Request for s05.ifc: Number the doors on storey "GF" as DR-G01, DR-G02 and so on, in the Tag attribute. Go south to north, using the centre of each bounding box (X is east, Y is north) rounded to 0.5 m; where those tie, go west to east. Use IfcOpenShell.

First a look at what the model holds.

```python
import ifcopenshell
import ifcopenshell.util.element
import ifcopenshell.util.placement

model = ifcopenshell.open("s05.ifc")
print(model.schema)
storey = next(s for s in model.by_type("IfcBuildingStorey") if s.Name == "GF")
doors = [e for e in ifcopenshell.util.element.get_decomposition(storey) if e.is_a("IfcDoor")]
for e in sorted(doors, key=lambda e: e.id()):
    origin = ifcopenshell.util.placement.get_local_placement(e.ObjectPlacement)[:3, 3]
    print(e.id(), e.Tag, e.Name, origin.round(2) + 0.0, sep=" | ")
```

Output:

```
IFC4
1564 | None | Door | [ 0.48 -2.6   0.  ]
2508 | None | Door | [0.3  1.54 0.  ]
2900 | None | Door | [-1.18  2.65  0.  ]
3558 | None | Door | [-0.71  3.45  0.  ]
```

```python
import ifcopenshell
import ifcopenshell.geom
import ifcopenshell.util.element
import ifcopenshell.util.shape

model = ifcopenshell.open("s05.ifc")
settings = ifcopenshell.geom.settings()
settings.set("use-world-coords", True)


def centre(element):
    shape = ifcopenshell.geom.create_shape(settings, element)
    return ifcopenshell.util.shape.get_bbox_centroid(shape.geometry)


storey = next(s for s in model.by_type("IfcBuildingStorey") if s.Name == "GF")
doors = [e for e in ifcopenshell.util.element.get_decomposition(storey) if e.is_a("IfcDoor")]

# Insertion points can sit at a corner or the storey origin, so sort by the geometry (in metres).
centres = {e: centre(e) for e in doors}
doors.sort(key=lambda e: (round(centres[e][1] / 0.5), centres[e][0]))

for i, e in enumerate(doors, start=1):
    number = f"DR-G{i:02d}"
    e.Tag = number
    print(e.id(), number)

model.write("s05_edited.ifc")
```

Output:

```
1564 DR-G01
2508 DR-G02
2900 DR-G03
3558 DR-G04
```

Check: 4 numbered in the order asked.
